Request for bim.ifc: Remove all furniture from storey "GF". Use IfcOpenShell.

First a look at what the model holds.

```python
import ifcopenshell
import ifcopenshell.util.element

model = ifcopenshell.open("bim.ifc")
print(model.schema)
storey = next(s for s in model.by_type("IfcBuildingStorey") if s.Name == "GF")
furniture = [e for e in ifcopenshell.util.element.get_decomposition(storey) if e.is_a("IfcFurnishingElement")]
seen = {}
for e in furniture:
    element_type = ifcopenshell.util.element.get_type(e)
    name = element_type.Name if element_type not in (None, e) else None
    seen[name] = seen.get(name, 0) + 1
for name, count in sorted(seen.items(), key=str):
    print(count, "x", name)
```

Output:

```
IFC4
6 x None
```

```python
import ifcopenshell
import ifcopenshell.api.root
import ifcopenshell.util.element

model = ifcopenshell.open("bim.ifc")

storey = next(s for s in model.by_type("IfcBuildingStorey") if s.Name == "GF")
furniture = [e for e in ifcopenshell.util.element.get_decomposition(storey) if e.is_a("IfcFurnishingElement")]

for e in furniture:
    ifcopenshell.api.root.remove_product(model, product=e)
print(len(furniture), "removed")

model.write("bim_rev.ifc")
```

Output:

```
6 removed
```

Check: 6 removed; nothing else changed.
